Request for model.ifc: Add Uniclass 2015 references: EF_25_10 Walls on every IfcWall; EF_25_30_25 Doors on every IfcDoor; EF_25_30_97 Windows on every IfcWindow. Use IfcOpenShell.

First a look at what the model holds.

```python
import ifcopenshell

model = ifcopenshell.open("model.ifc")
print(model.schema)
print("classifications:", [c.Name for c in model.by_type("IfcClassification")])
for ifc_class in ("IfcDoor", "IfcRoof", "IfcStair", "IfcWall", "IfcWindow"):
    print(ifc_class, len(model.by_type(ifc_class)))
```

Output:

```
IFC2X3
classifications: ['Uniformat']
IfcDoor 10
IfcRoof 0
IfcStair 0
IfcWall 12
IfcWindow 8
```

```python
import ifcopenshell
import ifcopenshell.api.classification

model = ifcopenshell.open("model.ifc")

# IFC2X3 requires Source and Edition and has no link from the project to the system.
system = model.create_entity("IfcClassification", Source="NBS", Edition="2015", Name="Uniclass 2015")

codes = {
    "IfcWall": ("EF_25_10", "Walls"),
    "IfcDoor": ("EF_25_30_25", "Doors"),
    "IfcWindow": ("EF_25_30_97", "Windows"),
}
for ifc_class, (code, name) in codes.items():
    products = model.by_type(ifc_class)
    ifcopenshell.api.classification.add_reference(
        model, products=products, classification=system, identification=code, name=name
    )
    print(code, len(products))

model.write("model-out.ifc")
```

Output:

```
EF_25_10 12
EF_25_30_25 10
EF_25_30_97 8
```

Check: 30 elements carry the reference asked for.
